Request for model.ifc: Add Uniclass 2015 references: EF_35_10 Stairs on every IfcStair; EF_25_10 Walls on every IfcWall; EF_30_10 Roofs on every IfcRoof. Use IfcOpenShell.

First a look at what the model holds.

```python
import ifcopenshell

model = ifcopenshell.open("model.ifc")
print(model.schema)
print("classifications:", [c.Name for c in model.by_type("IfcClassification")])
for ifc_class in ("IfcDoor", "IfcRoof", "IfcStair", "IfcWall", "IfcWindow"):
    print(ifc_class, len(model.by_type(ifc_class)))
```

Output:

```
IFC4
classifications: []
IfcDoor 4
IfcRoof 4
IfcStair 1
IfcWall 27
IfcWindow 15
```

```python
import ifcopenshell
import ifcopenshell.api.classification

model = ifcopenshell.open("model.ifc")

system = ifcopenshell.api.classification.add_classification(model, classification="Uniclass 2015")

codes = {
    "IfcStair": ("EF_35_10", "Stairs"),
    "IfcWall": ("EF_25_10", "Walls"),
    "IfcRoof": ("EF_30_10", "Roofs"),
}
for ifc_class, (code, name) in codes.items():
    products = model.by_type(ifc_class)
    ifcopenshell.api.classification.add_reference(
        model, products=products, classification=system, identification=code, name=name
    )
    print(code, len(products))

model.write("model_edited.ifc")
```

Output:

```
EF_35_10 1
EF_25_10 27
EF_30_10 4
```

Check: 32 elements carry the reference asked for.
